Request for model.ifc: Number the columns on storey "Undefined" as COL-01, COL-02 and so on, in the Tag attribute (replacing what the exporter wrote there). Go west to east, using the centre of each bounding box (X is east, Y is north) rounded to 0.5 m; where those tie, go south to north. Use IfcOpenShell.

First a look at what the model holds.

```python
import ifcopenshell
import ifcopenshell.util.element
import ifcopenshell.util.placement

model = ifcopenshell.open("model.ifc")
print(model.schema)
storey = next(s for s in model.by_type("IfcBuildingStorey") if s.Name == "Undefined")
columns = [e for e in ifcopenshell.util.element.get_decomposition(storey) if e.is_a("IfcColumn")]
for e in sorted(columns, key=lambda e: e.id()):
    origin = ifcopenshell.util.placement.get_local_placement(e.ObjectPlacement)[:3, 3]
    print(e.id(), e.Tag, e.Name, origin.round(2) + 0.0, sep=" | ")
```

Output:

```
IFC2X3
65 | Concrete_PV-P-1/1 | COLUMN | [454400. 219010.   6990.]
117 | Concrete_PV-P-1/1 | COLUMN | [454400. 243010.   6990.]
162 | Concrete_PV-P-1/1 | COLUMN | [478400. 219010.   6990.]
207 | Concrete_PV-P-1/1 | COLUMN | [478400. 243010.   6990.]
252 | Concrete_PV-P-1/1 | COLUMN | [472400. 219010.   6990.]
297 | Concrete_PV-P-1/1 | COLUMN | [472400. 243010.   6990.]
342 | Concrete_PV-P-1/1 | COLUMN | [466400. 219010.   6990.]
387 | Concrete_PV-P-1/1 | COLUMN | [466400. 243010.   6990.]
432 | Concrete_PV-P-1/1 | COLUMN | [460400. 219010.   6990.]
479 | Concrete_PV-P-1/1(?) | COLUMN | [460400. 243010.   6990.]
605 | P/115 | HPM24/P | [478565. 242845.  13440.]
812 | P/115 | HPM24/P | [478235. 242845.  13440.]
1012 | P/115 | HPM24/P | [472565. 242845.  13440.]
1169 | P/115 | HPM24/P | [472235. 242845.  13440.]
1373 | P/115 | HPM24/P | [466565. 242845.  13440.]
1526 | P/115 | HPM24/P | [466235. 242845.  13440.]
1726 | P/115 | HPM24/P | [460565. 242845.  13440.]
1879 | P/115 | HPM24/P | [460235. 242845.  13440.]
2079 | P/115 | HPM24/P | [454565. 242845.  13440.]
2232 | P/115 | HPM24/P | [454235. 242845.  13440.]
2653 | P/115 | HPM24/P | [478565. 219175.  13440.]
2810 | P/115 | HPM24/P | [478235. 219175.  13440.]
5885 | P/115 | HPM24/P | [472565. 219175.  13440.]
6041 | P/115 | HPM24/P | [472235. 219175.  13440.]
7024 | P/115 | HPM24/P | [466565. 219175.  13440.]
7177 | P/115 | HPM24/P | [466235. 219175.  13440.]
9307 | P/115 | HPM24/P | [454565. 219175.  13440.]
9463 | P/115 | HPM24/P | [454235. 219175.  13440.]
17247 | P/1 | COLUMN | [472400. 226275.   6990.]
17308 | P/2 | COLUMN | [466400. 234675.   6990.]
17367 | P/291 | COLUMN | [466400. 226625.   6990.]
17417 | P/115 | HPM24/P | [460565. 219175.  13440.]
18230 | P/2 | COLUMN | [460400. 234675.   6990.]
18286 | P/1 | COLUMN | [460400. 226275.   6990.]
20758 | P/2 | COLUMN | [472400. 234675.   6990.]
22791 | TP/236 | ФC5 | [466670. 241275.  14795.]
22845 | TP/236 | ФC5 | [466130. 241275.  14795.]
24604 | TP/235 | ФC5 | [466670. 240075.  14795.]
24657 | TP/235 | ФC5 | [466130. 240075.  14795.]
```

```python
import ifcopenshell
import ifcopenshell.geom
import ifcopenshell.util.element
import ifcopenshell.util.shape

model = ifcopenshell.open("model.ifc")
settings = ifcopenshell.geom.settings()
settings.set("use-world-coords", True)


def centre(element):
    shape = ifcopenshell.geom.create_shape(settings, element)
    return ifcopenshell.util.shape.get_bbox_centroid(shape.geometry)


storey = next(s for s in model.by_type("IfcBuildingStorey") if s.Name == "Undefined")
columns = [e for e in ifcopenshell.util.element.get_decomposition(storey) if e.is_a("IfcColumn")]

# Insertion points can sit at a corner or the storey origin, so sort by the geometry (in metres).
centres = {e: centre(e) for e in columns}
columns.sort(key=lambda e: (round(centres[e][0] / 0.5), centres[e][1]))

for i, e in enumerate(columns, start=1):
    number = f"COL-{i:02d}"
    e.Tag = number
    print(e.id(), number)

model.write("model_updated.ifc")
```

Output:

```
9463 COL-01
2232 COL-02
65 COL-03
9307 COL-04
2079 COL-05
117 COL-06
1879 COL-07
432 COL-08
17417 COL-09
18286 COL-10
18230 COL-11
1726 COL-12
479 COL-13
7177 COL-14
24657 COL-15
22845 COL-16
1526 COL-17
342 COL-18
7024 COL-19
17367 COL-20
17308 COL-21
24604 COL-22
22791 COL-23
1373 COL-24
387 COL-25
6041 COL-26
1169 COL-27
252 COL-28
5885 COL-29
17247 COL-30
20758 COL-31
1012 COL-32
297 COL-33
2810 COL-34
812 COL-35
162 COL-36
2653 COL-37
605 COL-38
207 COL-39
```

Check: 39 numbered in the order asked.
